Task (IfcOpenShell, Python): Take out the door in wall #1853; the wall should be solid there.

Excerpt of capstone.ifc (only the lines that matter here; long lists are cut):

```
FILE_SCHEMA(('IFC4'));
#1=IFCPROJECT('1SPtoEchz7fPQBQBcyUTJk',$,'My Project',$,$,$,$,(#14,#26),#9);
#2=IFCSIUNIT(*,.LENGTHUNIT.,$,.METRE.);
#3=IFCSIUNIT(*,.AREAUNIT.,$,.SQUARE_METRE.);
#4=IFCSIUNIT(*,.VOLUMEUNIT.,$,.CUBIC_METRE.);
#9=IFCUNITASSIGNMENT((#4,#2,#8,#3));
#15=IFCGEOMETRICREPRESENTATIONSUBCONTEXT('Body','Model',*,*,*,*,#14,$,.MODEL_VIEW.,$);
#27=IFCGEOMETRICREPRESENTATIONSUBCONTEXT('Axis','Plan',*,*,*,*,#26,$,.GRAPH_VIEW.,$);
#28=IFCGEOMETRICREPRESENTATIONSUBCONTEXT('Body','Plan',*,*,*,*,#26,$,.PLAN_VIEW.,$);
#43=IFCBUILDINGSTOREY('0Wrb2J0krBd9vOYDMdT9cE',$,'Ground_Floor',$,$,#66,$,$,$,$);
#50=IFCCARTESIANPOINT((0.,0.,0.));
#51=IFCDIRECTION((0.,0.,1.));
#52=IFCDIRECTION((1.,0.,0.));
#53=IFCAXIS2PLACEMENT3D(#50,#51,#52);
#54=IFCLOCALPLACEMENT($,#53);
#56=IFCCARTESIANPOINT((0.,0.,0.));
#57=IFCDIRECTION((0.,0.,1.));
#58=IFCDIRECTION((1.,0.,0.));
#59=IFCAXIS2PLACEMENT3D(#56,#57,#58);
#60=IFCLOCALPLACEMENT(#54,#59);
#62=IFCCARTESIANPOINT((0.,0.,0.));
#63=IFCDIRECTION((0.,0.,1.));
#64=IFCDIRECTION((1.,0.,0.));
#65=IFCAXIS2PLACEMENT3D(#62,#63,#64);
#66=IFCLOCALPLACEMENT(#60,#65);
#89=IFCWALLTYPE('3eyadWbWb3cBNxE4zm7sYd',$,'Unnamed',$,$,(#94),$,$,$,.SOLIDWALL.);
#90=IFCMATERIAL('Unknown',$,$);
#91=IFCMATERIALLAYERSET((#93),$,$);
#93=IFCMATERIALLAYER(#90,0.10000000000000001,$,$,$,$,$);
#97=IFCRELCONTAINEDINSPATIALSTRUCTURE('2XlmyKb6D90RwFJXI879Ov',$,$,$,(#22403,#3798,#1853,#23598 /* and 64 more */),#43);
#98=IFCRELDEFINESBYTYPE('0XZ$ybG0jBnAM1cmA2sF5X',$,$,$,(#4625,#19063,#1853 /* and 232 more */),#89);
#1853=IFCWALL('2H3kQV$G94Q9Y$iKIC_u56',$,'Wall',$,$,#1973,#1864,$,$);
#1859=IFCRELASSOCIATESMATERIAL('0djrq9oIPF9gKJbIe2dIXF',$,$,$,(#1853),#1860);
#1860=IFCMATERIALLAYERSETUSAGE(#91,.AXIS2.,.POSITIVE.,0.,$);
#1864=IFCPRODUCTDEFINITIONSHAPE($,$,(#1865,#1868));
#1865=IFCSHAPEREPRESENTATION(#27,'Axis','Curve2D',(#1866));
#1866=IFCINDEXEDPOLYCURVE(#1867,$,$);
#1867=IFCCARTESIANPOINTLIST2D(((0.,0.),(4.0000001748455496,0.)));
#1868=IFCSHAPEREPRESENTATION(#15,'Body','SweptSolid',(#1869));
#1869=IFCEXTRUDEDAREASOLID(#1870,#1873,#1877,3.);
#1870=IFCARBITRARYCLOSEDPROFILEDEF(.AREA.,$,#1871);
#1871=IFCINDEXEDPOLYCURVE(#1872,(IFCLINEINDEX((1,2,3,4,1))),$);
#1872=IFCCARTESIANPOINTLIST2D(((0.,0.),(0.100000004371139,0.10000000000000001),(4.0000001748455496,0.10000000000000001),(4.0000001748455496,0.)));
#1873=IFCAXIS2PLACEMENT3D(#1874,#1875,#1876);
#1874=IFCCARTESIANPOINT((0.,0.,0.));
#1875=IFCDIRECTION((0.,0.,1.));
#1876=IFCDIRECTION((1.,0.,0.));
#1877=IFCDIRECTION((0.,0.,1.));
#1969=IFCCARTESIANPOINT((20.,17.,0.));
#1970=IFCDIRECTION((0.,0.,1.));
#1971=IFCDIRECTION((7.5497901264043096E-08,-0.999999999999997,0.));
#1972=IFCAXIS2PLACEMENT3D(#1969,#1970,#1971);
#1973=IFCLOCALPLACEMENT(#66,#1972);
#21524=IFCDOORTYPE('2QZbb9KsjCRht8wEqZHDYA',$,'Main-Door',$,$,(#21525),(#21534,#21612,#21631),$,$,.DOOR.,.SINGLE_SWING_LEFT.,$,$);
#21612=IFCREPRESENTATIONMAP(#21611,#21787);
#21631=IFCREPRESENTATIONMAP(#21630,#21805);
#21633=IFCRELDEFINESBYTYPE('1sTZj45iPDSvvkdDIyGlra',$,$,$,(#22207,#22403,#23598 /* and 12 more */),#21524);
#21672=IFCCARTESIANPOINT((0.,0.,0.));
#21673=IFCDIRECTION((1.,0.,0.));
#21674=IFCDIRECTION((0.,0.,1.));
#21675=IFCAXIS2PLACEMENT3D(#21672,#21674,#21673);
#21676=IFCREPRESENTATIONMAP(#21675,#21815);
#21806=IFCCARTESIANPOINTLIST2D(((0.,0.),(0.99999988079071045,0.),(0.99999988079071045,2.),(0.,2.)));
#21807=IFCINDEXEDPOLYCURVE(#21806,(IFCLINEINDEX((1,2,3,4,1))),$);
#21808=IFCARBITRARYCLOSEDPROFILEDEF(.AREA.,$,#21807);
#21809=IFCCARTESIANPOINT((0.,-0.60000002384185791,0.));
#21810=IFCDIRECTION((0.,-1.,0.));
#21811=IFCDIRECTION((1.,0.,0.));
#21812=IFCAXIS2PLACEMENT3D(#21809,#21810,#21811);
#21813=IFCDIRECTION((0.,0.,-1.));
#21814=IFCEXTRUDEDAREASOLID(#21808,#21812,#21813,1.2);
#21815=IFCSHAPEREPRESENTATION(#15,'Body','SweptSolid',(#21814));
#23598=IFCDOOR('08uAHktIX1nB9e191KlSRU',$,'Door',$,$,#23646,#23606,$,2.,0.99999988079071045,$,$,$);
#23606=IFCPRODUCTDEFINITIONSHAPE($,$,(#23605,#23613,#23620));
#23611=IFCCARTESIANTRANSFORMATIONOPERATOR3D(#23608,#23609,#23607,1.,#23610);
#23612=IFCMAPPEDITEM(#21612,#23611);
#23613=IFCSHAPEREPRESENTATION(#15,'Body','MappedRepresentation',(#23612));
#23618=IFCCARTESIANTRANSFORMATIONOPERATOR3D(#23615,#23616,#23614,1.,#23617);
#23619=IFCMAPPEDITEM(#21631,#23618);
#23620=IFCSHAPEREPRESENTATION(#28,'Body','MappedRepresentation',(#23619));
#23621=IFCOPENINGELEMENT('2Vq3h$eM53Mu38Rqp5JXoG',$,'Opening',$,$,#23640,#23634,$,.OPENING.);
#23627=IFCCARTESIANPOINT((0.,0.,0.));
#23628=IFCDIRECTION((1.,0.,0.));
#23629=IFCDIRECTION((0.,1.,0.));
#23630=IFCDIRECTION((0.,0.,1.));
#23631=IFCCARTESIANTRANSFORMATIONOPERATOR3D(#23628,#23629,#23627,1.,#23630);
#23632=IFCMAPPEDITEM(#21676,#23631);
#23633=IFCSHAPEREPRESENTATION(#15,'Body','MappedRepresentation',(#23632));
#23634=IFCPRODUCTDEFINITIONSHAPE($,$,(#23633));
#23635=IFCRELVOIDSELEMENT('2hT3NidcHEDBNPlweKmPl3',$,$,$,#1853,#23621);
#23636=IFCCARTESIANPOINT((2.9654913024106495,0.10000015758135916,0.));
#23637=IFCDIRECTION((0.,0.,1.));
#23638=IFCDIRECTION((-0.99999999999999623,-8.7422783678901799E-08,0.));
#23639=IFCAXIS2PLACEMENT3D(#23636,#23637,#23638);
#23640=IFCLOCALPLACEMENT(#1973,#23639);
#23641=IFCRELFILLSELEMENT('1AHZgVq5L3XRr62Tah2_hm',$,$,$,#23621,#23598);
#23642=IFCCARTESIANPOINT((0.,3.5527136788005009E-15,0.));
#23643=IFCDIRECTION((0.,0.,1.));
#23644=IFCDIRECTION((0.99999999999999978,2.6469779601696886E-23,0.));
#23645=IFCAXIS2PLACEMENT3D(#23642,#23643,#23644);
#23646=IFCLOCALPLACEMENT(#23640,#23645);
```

```python
import ifcopenshell
import ifcopenshell.api.feature
import ifcopenshell.api.root
import ifcopenshell.geom
import ifcopenshell.util.shape

model = ifcopenshell.open("capstone.ifc")
settings = ifcopenshell.geom.settings()


def volume(element):
    """Net volume in cubic metres, openings subtracted."""
    shape = ifcopenshell.geom.create_shape(settings, element)
    return ifcopenshell.util.shape.get_volume(shape.geometry)


door = model.by_id(23598)
opening = door.FillsVoids[0].RelatingOpeningElement
wall = opening.VoidsElements[0].RelatingBuildingElement
before = volume(wall)

ifcopenshell.api.root.remove_product(model, product=door)
ifcopenshell.api.feature.remove_feature(model, feature=opening)

after = volume(wall)

print(f"wall volume {before:.3f} -> {after:.3f} m3")

model.write("capstone_rev.ifc")
```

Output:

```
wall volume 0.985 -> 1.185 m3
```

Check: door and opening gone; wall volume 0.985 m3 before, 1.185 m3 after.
